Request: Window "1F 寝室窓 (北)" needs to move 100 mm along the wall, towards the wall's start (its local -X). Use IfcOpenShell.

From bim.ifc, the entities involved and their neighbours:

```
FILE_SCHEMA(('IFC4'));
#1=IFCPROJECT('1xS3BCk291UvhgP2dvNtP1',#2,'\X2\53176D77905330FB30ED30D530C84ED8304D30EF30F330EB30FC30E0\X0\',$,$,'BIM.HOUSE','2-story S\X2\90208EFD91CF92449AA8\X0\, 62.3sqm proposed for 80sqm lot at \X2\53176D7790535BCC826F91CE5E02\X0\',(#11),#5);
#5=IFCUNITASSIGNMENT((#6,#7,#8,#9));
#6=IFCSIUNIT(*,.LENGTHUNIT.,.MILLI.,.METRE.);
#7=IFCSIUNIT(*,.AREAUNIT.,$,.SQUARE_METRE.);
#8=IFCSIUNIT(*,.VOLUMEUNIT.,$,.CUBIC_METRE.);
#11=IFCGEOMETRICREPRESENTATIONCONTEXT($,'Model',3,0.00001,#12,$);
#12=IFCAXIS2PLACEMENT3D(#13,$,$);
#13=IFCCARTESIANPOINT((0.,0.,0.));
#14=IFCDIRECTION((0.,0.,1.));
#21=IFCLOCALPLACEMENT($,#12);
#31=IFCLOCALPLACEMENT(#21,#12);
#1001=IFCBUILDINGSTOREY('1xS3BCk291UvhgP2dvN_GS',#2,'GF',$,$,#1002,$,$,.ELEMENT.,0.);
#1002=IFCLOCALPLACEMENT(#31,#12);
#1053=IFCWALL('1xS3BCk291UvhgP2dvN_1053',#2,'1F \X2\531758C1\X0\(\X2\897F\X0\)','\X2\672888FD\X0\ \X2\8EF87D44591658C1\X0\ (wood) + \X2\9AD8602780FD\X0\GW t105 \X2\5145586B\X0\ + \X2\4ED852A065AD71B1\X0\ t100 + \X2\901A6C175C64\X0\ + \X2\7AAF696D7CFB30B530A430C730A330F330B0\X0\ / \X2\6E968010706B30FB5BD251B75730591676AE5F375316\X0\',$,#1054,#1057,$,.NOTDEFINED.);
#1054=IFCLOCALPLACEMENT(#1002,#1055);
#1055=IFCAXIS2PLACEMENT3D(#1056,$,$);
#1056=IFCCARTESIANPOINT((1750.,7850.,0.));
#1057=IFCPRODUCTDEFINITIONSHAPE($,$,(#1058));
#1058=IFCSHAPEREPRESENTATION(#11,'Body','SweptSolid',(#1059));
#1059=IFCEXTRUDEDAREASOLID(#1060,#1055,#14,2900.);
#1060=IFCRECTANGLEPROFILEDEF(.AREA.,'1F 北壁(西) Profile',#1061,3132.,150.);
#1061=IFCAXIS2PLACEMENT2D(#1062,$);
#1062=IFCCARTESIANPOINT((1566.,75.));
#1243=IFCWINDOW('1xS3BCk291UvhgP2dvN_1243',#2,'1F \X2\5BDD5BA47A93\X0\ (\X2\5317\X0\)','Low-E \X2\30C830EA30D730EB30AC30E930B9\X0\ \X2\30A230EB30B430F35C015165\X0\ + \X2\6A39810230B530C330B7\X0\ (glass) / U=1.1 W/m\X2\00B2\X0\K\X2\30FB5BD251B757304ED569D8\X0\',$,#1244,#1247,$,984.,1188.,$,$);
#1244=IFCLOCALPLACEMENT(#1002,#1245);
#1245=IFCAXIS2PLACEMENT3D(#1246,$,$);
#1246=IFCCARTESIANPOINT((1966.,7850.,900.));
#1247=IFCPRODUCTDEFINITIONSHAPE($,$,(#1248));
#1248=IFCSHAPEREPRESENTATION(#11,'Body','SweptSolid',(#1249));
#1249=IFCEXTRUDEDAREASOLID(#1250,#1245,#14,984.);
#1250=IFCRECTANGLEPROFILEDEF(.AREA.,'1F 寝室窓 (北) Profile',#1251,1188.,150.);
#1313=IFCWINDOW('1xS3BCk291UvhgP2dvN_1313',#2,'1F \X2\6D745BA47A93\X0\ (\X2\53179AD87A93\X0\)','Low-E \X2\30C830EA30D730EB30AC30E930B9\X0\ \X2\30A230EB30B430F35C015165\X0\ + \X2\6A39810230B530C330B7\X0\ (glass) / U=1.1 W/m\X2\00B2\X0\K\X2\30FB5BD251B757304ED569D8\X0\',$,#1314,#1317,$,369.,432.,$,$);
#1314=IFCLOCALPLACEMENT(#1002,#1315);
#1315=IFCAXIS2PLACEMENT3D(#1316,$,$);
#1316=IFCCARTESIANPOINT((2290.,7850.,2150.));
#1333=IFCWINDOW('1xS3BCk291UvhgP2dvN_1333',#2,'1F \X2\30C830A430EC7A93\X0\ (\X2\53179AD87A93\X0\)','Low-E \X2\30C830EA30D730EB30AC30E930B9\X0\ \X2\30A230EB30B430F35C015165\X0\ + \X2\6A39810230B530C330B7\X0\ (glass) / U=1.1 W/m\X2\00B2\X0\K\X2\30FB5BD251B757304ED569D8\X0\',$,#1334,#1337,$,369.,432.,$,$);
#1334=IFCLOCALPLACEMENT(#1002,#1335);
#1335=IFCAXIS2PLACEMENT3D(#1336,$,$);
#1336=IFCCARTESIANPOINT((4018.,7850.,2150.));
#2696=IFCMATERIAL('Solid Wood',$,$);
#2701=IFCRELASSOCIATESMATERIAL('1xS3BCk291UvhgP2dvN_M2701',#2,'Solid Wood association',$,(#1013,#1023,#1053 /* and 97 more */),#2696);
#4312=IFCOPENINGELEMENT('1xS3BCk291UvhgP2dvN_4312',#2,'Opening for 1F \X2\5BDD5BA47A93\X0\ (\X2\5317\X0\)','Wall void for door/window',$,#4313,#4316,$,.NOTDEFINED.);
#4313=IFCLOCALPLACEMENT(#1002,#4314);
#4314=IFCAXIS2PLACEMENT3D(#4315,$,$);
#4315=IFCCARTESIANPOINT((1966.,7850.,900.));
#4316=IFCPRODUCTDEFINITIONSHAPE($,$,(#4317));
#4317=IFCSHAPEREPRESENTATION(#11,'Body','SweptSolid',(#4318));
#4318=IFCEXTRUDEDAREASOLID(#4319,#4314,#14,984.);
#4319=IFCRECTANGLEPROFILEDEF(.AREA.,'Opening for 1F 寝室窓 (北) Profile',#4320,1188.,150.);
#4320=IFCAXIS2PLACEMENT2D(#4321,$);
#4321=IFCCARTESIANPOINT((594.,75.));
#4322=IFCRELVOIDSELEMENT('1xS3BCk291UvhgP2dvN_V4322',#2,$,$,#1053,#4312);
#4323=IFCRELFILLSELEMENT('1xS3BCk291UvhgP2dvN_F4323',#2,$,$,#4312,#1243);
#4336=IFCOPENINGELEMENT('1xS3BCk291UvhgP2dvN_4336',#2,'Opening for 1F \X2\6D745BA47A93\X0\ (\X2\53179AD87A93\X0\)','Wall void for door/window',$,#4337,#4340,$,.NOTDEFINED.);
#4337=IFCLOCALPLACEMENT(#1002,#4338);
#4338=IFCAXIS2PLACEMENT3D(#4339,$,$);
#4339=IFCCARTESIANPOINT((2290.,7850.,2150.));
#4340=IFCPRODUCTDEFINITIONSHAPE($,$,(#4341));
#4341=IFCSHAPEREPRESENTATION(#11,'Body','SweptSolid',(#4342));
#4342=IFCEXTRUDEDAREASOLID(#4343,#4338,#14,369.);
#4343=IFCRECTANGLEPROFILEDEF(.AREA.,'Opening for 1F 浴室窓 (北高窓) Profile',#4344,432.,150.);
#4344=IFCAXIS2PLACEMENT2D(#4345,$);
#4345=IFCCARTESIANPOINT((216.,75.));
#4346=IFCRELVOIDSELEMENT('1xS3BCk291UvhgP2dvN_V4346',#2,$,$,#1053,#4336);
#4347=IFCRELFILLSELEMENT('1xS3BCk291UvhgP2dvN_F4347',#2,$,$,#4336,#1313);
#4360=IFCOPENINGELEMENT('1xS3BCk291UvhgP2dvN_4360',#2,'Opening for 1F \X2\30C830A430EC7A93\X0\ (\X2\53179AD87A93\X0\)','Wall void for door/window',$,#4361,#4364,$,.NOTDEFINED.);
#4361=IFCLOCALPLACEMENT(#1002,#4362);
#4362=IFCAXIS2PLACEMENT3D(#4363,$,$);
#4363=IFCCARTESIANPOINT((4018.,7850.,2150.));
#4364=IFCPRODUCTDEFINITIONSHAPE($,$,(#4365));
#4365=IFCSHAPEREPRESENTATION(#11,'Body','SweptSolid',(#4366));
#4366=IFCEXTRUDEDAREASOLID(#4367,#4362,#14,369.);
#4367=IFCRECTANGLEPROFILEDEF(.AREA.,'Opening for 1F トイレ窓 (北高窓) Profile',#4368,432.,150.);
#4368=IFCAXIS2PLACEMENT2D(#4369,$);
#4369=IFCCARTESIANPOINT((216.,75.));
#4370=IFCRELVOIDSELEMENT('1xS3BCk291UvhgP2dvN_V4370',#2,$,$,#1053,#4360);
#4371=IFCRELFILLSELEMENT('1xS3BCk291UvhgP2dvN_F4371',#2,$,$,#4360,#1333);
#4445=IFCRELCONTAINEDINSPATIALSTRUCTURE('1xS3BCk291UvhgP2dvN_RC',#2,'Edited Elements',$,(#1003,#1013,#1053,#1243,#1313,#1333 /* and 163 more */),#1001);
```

```python
import ifcopenshell
import ifcopenshell.api.geometry
import ifcopenshell.util.placement
import ifcopenshell.util.unit

model = ifcopenshell.open("bim.ifc")
unit_scale = ifcopenshell.util.unit.calculate_unit_scale(model)

window = model.by_guid("1xS3BCk291UvhgP2dvN_1243")
opening = window.FillsVoids[0].RelatingOpeningElement
wall = opening.VoidsElements[0].RelatingBuildingElement

wall_matrix = ifcopenshell.util.placement.get_local_placement(wall.ObjectPlacement)
shift = wall_matrix[:3, 0] * -0.1 / unit_scale
before = ifcopenshell.util.placement.get_local_placement(window.ObjectPlacement)[:3, 3].copy()

# The window is not placed relative to its opening, so move both.
for product in (opening, window):
    matrix = ifcopenshell.util.placement.get_local_placement(product.ObjectPlacement)
    matrix[:3, 3] += shift
    ifcopenshell.api.geometry.edit_object_placement(model, product=product, matrix=matrix, is_si=False)

after = ifcopenshell.util.placement.get_local_placement(window.ObjectPlacement)[:3, 3]
print("window moved by", (after - before).round(3) + 0.0)

model.write("bim_updated.ifc")
```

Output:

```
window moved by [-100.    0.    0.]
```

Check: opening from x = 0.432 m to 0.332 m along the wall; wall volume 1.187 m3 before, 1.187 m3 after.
